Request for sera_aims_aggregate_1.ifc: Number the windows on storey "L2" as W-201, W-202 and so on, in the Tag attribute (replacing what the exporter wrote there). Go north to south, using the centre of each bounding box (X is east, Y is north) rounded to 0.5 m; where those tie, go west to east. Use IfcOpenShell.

First a look at what the model holds.

```python
import ifcopenshell
import ifcopenshell.util.element
import ifcopenshell.util.placement

model = ifcopenshell.open("sera_aims_aggregate_1.ifc")
print(model.schema)
storey = next(s for s in model.by_type("IfcBuildingStorey") if s.Name == "L2")
windows = [e for e in ifcopenshell.util.element.get_decomposition(storey) if e.is_a("IfcWindow")]
for e in sorted(windows, key=lambda e: e.id()):
    origin = ifcopenshell.util.placement.get_local_placement(e.ObjectPlacement)[:3, 3]
    print(e.id(), e.Tag, e.Name, origin.round(2) + 0.0, sep=" | ")
```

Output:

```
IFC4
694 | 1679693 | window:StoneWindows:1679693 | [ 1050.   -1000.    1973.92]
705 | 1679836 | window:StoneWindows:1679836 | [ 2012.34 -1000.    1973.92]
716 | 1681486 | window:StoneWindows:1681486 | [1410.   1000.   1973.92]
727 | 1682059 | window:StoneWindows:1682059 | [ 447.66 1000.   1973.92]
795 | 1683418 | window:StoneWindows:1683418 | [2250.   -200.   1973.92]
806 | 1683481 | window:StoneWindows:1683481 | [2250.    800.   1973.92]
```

```python
import ifcopenshell
import ifcopenshell.geom
import ifcopenshell.util.element
import ifcopenshell.util.shape

model = ifcopenshell.open("sera_aims_aggregate_1.ifc")
settings = ifcopenshell.geom.settings()
settings.set("use-world-coords", True)


def centre(element):
    shape = ifcopenshell.geom.create_shape(settings, element)
    return ifcopenshell.util.shape.get_bbox_centroid(shape.geometry)


storey = next(s for s in model.by_type("IfcBuildingStorey") if s.Name == "L2")
windows = [e for e in ifcopenshell.util.element.get_decomposition(storey) if e.is_a("IfcWindow")]

# Insertion points can sit at a corner or the storey origin, so sort by the geometry (in metres).
centres = {e: centre(e) for e in windows}
windows.sort(key=lambda e: (-round(centres[e][1] / 0.5), centres[e][0]))

for i, e in enumerate(windows, start=1):
    number = f"W-2{i:02d}"
    e.Tag = number
    print(e.id(), number)

model.write("sera_aims_aggregate_1_v2.ifc")
```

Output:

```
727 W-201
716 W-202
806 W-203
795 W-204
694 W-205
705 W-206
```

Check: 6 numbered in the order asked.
